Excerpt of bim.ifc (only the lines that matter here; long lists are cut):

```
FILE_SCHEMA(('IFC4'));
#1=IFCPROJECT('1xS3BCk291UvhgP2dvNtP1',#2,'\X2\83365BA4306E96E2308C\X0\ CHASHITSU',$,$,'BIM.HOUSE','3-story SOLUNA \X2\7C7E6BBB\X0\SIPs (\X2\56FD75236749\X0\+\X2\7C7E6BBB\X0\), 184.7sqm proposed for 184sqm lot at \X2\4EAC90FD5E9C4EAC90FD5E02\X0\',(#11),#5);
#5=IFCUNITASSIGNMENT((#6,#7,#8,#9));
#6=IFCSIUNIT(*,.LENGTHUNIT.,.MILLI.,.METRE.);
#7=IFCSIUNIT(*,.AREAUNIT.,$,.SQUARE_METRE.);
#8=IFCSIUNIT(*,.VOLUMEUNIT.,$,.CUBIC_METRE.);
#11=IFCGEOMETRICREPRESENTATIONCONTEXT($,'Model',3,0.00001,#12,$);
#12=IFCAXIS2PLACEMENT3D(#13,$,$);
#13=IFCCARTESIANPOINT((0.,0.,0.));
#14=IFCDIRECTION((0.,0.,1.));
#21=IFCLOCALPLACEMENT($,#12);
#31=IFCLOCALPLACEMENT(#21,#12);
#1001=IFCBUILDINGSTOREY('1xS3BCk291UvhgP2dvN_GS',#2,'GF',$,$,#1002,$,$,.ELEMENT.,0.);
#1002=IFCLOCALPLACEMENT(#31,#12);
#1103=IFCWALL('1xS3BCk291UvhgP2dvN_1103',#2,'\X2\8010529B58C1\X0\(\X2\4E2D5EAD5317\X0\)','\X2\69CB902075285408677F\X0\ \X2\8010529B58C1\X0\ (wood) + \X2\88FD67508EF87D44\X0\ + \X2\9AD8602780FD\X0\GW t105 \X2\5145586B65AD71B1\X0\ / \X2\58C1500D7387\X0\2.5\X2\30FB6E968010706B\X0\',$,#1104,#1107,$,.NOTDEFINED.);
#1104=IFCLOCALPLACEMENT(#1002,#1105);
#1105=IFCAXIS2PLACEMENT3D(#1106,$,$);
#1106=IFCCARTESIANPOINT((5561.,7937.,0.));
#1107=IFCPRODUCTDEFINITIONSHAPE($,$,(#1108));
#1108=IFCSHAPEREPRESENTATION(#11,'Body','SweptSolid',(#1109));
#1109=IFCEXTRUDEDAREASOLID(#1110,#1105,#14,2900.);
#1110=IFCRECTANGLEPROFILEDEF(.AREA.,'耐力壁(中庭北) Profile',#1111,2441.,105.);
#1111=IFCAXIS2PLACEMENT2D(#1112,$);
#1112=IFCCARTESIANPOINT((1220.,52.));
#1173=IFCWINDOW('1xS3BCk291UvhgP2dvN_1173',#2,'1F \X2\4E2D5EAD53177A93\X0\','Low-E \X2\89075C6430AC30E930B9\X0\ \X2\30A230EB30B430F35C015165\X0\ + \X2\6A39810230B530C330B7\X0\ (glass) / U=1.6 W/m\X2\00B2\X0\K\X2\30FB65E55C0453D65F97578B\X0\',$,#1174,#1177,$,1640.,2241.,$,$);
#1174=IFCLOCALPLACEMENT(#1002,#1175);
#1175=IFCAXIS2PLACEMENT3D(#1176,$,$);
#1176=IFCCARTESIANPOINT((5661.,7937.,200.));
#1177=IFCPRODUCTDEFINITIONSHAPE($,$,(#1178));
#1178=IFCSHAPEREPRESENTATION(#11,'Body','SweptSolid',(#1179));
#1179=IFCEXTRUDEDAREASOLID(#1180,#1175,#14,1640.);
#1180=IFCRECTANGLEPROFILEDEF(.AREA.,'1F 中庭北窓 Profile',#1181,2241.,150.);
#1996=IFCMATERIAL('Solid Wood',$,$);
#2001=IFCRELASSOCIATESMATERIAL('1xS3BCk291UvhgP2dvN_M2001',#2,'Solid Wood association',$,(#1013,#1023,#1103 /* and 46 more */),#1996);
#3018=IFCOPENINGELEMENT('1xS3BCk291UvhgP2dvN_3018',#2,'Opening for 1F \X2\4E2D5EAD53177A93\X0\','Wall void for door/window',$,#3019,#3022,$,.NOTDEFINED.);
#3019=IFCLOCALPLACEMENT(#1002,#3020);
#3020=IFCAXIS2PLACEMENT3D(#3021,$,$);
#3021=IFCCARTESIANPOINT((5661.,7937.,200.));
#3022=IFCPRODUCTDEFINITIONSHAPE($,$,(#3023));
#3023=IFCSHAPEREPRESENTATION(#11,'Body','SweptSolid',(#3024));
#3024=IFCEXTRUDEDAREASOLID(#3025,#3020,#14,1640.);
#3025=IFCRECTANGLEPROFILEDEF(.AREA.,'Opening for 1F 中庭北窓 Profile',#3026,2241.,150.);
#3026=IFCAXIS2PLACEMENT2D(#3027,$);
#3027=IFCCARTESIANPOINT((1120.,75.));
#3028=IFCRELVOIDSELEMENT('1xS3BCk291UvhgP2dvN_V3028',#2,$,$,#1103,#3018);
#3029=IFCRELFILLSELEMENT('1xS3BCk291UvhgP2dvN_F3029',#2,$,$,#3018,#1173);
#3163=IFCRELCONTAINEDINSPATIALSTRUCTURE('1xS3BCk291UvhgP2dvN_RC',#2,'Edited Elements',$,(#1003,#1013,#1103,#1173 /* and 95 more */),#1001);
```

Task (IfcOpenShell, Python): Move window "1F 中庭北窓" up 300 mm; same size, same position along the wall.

```python
import numpy as np
import ifcopenshell
import ifcopenshell.api.geometry
import ifcopenshell.util.placement
import ifcopenshell.util.unit

model = ifcopenshell.open("bim.ifc")
unit_scale = ifcopenshell.util.unit.calculate_unit_scale(model)

window = model.by_guid("1xS3BCk291UvhgP2dvN_1173")
opening = window.FillsVoids[0].RelatingOpeningElement
dz = 300.0

shift = np.array([0.0, 0.0, dz])
# The window is not placed relative to its opening, so move both.
for product in (opening, window):
    matrix = ifcopenshell.util.placement.get_local_placement(product.ObjectPlacement)
    matrix[:3, 3] += shift
    ifcopenshell.api.geometry.edit_object_placement(model, product=product, matrix=matrix, is_si=False)

print(f"moved by {dz * unit_scale:+.3f} m")

model.write("bim_rev.ifc")
```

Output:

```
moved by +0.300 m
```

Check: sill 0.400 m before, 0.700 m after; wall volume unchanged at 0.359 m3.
